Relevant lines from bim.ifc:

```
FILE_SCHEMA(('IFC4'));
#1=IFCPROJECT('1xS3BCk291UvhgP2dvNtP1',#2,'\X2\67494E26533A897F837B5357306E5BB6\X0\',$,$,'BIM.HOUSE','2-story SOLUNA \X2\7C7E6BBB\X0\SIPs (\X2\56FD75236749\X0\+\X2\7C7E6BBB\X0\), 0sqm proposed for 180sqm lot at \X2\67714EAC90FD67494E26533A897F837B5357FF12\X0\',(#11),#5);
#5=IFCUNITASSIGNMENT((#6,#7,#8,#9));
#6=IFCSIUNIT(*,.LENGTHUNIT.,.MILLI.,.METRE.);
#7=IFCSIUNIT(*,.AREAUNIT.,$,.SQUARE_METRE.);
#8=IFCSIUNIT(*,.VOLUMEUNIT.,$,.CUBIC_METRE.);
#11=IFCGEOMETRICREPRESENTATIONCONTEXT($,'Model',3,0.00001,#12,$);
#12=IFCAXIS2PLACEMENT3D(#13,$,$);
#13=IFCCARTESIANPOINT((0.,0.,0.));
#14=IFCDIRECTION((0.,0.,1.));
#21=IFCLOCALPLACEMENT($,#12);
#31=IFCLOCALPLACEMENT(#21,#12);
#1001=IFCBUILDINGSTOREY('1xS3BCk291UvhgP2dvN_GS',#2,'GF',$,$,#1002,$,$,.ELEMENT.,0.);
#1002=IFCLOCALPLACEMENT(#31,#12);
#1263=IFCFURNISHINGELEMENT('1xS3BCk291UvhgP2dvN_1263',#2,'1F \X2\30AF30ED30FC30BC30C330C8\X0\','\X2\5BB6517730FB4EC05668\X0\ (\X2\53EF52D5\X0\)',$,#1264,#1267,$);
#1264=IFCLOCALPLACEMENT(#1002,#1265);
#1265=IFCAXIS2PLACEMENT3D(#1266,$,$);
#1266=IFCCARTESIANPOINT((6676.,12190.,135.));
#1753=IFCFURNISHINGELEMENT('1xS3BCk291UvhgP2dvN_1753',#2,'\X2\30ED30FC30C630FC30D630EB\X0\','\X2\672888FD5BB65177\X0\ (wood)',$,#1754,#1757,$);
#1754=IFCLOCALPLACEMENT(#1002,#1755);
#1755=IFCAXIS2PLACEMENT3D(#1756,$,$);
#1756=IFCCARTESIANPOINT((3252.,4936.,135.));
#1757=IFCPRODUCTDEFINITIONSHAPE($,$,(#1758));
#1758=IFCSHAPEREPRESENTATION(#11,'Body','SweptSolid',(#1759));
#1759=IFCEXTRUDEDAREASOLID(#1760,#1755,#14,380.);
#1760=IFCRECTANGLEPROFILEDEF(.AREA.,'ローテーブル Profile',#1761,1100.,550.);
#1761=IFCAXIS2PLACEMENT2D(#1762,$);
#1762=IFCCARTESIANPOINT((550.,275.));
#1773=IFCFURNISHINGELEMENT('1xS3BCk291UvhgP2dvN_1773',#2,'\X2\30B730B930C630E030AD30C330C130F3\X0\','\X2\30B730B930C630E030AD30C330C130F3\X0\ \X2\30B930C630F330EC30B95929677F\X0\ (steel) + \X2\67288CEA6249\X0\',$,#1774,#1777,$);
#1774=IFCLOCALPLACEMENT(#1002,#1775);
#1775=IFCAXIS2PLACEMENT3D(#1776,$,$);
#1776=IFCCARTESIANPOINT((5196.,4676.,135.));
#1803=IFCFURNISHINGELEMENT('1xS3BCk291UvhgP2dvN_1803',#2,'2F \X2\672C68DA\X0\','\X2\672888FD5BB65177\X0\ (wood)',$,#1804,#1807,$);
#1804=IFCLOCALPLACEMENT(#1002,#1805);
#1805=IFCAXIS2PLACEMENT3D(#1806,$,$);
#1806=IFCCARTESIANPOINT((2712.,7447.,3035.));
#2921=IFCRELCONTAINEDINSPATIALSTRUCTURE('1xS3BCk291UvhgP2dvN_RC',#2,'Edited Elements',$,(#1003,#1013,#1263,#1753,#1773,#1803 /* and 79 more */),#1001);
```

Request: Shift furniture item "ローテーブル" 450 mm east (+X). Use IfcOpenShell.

```python
import ifcopenshell
import ifcopenshell.api.geometry
import ifcopenshell.util.placement
import ifcopenshell.util.unit

model = ifcopenshell.open("bim.ifc")
unit_scale = ifcopenshell.util.unit.calculate_unit_scale(model)

item = model.by_guid("1xS3BCk291UvhgP2dvN_1753")
matrix = ifcopenshell.util.placement.get_local_placement(item.ObjectPlacement)
matrix[0, 3] += 0.45 / unit_scale
ifcopenshell.api.geometry.edit_object_placement(model, product=item, matrix=matrix, is_si=False)

print(ifcopenshell.util.placement.get_local_placement(item.ObjectPlacement).round(3) + 0.0)

model.write("bim_updated.ifc")
```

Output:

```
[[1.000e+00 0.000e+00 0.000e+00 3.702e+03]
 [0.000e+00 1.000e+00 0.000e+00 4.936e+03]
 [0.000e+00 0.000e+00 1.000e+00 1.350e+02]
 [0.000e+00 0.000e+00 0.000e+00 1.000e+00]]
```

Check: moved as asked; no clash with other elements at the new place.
